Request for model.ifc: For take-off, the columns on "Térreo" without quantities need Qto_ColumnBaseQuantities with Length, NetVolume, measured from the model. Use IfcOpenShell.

First a look at what the model holds.

```python
import ifcopenshell
import ifcopenshell.util.element
import ifcopenshell.util.unit

model = ifcopenshell.open("model.ifc")
print(model.schema)
for unit_type in ("LENGTHUNIT", "AREAUNIT", "VOLUMEUNIT"):
    print(unit_type, ifcopenshell.util.unit.calculate_unit_scale(model, unit_type))
storey = next(s for s in model.by_type("IfcBuildingStorey") if s.Name == "Térreo")
columns = [e for e in ifcopenshell.util.element.get_decomposition(storey) if e.is_a("IfcColumn")]
for e in sorted(columns, key=lambda e: e.id()):
    print(e.id(), e.is_a(), e.Name, list(ifcopenshell.util.element.get_psets(e, qtos_only=True)), sep=" | ")
```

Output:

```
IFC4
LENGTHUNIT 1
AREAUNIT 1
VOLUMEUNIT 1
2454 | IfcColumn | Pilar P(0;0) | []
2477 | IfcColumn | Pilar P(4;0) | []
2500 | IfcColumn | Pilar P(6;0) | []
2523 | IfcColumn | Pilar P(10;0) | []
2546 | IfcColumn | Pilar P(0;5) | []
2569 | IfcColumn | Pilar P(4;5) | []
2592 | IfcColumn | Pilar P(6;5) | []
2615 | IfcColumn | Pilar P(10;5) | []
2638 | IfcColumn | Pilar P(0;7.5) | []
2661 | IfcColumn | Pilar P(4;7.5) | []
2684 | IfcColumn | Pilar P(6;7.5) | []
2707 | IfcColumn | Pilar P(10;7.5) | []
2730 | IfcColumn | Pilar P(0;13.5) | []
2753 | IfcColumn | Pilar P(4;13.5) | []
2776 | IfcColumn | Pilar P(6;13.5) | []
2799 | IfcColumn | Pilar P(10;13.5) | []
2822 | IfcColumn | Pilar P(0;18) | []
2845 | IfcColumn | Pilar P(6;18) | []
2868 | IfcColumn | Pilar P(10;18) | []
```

```python
import ifcopenshell
import ifcopenshell.api.pset
import ifcopenshell.geom
import ifcopenshell.util.element
import ifcopenshell.util.shape
import ifcopenshell.util.unit

model = ifcopenshell.open("model.ifc")
unit_scale = ifcopenshell.util.unit.calculate_unit_scale(model)
volume_scale = ifcopenshell.util.unit.calculate_unit_scale(model, "VOLUMEUNIT")
settings = ifcopenshell.geom.settings()

storey = next(s for s in model.by_type("IfcBuildingStorey") if s.Name == "Térreo")
columns = [e for e in ifcopenshell.util.element.get_decomposition(storey) if e.is_a("IfcColumn")]

for e in sorted(columns, key=lambda e: e.id()):
    if ifcopenshell.util.element.get_psets(e, qtos_only=True, should_inherit=False):
        continue
    # Geometry comes back in metres, in the element's own axes.
    shape = ifcopenshell.geom.create_shape(settings, e)
    values = {
        "Length": ifcopenshell.util.shape.get_z(shape.geometry) / unit_scale,
        "NetVolume": ifcopenshell.util.shape.get_volume(shape.geometry) / volume_scale,
    }
    qto = ifcopenshell.api.pset.add_qto(model, product=e, name="Qto_ColumnBaseQuantities")
    ifcopenshell.api.pset.edit_qto(model, qto=qto, properties=values)
    print(e.id(), {k: round(v, 3) for k, v in values.items()})

model.write("model-out.ifc")
```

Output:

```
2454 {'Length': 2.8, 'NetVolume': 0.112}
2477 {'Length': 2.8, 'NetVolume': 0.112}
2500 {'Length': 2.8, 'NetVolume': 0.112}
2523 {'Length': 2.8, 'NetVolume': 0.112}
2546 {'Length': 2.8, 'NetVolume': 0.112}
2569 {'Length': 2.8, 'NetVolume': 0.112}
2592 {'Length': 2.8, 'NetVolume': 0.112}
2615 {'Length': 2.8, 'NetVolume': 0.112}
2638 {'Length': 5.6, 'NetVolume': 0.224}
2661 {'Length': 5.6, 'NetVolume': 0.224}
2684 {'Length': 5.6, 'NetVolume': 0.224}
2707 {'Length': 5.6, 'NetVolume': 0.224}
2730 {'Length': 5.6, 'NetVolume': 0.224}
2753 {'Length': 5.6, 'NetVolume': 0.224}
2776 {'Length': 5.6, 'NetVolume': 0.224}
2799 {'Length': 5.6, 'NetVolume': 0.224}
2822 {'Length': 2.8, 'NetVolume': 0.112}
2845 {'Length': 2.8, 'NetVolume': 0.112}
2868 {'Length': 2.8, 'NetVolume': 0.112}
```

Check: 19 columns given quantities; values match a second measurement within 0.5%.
